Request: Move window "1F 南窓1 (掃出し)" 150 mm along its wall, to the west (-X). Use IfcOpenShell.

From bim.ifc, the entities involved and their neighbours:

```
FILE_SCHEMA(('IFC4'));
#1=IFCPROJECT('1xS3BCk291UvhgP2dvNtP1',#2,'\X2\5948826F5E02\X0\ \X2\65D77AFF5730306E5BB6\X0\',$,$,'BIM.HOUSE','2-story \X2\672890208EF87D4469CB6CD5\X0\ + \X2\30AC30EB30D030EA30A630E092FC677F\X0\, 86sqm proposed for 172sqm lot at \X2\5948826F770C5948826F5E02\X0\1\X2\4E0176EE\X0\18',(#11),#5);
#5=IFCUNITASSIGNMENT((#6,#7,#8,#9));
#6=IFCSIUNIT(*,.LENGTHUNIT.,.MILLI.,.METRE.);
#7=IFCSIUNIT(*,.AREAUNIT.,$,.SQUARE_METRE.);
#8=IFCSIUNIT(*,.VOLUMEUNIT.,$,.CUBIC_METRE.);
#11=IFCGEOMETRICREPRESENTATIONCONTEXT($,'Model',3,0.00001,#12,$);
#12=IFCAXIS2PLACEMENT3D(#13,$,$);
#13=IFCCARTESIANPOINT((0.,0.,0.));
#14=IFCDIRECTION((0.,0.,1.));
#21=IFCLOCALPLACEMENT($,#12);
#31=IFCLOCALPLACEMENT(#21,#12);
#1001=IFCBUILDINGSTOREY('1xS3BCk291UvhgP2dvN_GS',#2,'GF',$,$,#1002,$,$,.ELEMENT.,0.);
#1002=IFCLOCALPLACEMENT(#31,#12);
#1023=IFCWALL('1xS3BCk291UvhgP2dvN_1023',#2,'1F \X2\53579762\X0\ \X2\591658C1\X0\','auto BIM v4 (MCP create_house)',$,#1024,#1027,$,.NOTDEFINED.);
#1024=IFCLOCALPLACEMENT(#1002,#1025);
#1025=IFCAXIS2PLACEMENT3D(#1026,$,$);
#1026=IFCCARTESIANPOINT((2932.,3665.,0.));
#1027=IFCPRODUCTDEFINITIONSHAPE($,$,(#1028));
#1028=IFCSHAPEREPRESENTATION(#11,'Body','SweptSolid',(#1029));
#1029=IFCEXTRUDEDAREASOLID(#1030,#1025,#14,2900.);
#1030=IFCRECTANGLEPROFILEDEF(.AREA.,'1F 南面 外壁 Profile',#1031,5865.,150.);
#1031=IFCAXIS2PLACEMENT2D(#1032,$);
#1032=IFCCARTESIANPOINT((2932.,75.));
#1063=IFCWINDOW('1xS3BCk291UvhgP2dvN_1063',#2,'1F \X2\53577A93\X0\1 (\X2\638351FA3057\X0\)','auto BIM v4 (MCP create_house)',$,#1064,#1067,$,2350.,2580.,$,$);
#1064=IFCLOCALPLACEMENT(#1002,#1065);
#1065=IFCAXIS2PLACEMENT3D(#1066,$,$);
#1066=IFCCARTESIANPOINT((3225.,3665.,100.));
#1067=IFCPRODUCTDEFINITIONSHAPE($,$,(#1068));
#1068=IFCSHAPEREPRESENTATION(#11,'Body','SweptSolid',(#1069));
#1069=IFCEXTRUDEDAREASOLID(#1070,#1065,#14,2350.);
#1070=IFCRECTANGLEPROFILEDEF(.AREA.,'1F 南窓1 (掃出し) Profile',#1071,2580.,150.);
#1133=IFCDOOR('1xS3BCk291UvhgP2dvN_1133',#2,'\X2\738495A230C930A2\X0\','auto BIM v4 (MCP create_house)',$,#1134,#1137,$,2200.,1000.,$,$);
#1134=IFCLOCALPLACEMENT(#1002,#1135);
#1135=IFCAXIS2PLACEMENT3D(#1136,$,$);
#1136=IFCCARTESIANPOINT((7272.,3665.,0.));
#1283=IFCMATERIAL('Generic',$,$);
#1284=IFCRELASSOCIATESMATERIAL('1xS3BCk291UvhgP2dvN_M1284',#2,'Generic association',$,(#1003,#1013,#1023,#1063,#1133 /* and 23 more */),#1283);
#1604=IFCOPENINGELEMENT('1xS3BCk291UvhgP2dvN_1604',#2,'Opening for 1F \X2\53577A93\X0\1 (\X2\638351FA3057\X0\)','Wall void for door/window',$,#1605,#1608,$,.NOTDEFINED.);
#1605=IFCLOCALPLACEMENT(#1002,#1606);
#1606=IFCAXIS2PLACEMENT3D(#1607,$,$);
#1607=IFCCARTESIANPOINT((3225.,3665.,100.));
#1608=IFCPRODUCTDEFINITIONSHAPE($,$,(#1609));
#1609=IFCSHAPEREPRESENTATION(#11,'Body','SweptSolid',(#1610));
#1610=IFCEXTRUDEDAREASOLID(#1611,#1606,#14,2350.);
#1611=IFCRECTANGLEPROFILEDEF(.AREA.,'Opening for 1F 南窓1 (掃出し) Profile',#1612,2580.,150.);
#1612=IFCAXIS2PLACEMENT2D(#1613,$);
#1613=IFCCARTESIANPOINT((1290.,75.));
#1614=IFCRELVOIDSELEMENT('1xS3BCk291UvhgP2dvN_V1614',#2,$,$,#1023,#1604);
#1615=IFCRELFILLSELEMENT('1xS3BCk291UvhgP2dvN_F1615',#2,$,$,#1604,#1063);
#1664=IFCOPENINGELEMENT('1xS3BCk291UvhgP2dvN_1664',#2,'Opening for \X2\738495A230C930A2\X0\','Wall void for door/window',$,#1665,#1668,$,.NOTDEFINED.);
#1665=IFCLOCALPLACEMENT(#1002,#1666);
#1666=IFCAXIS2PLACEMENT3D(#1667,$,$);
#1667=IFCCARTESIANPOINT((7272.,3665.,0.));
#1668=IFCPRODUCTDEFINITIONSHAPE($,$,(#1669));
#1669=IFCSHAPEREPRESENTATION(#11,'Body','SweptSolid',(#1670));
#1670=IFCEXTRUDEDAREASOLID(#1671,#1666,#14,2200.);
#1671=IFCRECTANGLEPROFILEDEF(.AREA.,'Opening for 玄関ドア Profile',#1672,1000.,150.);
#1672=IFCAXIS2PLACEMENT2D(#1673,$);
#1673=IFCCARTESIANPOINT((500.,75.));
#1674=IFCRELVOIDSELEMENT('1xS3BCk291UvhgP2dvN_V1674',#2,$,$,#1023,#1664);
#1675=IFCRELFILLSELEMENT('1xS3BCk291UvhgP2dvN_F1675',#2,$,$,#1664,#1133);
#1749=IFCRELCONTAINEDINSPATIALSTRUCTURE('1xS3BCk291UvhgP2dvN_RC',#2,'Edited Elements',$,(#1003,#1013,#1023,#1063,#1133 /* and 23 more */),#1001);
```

```python
import ifcopenshell
import ifcopenshell.api.geometry
import ifcopenshell.util.placement

model = ifcopenshell.open("bim.ifc")

window = model.by_id(1063)
opening = window.FillsVoids[0].RelatingOpeningElement
wall = opening.VoidsElements[0].RelatingBuildingElement

wall_matrix = ifcopenshell.util.placement.get_local_placement(wall.ObjectPlacement)
shift = wall_matrix[:3, 0] * -150.0
before = ifcopenshell.util.placement.get_local_placement(window.ObjectPlacement)[:3, 3].copy()

# The window is not placed relative to its opening, so move both.
for product in (opening, window):
    matrix = ifcopenshell.util.placement.get_local_placement(product.ObjectPlacement)
    matrix[:3, 3] += shift
    ifcopenshell.api.geometry.edit_object_placement(model, product=product, matrix=matrix, is_si=False)

after = ifcopenshell.util.placement.get_local_placement(window.ObjectPlacement)[:3, 3]
print("window moved by", (after - before).round(3) + 0.0)

model.write("bim_v2.ifc")
```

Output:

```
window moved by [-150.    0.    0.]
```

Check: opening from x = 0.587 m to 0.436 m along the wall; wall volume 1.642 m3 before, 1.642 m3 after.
